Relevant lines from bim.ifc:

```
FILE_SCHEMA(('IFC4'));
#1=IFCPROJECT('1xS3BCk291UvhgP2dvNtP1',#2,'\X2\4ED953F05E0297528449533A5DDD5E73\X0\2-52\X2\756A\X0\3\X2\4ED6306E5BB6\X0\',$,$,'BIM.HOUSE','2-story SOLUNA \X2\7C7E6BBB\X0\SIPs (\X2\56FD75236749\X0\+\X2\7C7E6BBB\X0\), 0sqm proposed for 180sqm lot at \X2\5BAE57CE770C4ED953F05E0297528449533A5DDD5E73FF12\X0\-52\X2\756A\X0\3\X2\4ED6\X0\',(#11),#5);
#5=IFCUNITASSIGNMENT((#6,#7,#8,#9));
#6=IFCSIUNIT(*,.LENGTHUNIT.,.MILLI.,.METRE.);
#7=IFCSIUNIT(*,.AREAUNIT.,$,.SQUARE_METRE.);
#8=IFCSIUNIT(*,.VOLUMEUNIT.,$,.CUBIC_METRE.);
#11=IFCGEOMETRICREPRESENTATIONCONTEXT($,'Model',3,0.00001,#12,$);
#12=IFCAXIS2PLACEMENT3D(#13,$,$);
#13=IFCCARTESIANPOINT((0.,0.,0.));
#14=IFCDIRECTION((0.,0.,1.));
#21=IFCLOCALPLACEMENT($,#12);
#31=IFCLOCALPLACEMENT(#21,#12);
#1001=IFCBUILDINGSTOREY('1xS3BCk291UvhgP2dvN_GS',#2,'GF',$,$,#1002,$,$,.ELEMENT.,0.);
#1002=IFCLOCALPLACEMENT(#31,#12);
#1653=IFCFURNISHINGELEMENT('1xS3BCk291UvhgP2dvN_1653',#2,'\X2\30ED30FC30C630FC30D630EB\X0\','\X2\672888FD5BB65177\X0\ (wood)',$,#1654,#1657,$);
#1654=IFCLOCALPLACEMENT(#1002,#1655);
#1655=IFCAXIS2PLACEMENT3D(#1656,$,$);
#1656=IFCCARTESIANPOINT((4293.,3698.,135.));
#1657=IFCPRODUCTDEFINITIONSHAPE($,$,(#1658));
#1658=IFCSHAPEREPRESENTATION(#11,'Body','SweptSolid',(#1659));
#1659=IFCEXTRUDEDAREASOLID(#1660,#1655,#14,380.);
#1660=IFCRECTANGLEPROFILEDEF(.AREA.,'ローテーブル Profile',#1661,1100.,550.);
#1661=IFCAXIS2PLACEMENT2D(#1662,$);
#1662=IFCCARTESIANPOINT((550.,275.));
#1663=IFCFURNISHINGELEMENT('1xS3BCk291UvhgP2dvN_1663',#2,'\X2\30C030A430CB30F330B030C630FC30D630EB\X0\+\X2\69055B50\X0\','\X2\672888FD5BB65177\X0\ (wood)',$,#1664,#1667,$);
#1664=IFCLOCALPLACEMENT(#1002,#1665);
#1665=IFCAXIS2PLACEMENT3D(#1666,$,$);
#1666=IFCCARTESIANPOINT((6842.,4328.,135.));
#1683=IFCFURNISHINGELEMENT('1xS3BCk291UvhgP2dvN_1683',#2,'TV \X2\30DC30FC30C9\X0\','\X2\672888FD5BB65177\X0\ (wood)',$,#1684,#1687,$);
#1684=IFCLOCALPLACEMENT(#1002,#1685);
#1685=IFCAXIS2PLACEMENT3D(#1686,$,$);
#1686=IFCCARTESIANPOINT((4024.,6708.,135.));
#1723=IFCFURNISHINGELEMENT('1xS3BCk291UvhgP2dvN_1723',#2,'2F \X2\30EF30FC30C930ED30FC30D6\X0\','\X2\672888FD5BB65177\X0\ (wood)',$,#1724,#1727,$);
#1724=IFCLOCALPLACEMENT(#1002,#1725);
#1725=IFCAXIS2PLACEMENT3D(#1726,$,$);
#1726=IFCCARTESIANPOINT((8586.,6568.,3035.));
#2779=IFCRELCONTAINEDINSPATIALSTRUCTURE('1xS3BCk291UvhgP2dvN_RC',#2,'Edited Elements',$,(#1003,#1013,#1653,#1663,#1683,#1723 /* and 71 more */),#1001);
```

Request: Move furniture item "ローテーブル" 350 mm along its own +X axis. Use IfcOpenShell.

```python
import ifcopenshell
import ifcopenshell.api.geometry
import ifcopenshell.util.placement

model = ifcopenshell.open("bim.ifc")

item = model.by_guid("1xS3BCk291UvhgP2dvN_1653")
matrix = ifcopenshell.util.placement.get_local_placement(item.ObjectPlacement)
matrix[:3, 3] += matrix[:3, 0] * 350.0
ifcopenshell.api.geometry.edit_object_placement(model, product=item, matrix=matrix, is_si=False)

print(ifcopenshell.util.placement.get_local_placement(item.ObjectPlacement).round(3) + 0.0)

model.write("bim_rev.ifc")
```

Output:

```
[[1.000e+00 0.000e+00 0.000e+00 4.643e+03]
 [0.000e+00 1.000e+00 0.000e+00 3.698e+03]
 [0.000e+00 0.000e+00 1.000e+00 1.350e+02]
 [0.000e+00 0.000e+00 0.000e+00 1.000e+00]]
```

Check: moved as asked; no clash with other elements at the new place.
